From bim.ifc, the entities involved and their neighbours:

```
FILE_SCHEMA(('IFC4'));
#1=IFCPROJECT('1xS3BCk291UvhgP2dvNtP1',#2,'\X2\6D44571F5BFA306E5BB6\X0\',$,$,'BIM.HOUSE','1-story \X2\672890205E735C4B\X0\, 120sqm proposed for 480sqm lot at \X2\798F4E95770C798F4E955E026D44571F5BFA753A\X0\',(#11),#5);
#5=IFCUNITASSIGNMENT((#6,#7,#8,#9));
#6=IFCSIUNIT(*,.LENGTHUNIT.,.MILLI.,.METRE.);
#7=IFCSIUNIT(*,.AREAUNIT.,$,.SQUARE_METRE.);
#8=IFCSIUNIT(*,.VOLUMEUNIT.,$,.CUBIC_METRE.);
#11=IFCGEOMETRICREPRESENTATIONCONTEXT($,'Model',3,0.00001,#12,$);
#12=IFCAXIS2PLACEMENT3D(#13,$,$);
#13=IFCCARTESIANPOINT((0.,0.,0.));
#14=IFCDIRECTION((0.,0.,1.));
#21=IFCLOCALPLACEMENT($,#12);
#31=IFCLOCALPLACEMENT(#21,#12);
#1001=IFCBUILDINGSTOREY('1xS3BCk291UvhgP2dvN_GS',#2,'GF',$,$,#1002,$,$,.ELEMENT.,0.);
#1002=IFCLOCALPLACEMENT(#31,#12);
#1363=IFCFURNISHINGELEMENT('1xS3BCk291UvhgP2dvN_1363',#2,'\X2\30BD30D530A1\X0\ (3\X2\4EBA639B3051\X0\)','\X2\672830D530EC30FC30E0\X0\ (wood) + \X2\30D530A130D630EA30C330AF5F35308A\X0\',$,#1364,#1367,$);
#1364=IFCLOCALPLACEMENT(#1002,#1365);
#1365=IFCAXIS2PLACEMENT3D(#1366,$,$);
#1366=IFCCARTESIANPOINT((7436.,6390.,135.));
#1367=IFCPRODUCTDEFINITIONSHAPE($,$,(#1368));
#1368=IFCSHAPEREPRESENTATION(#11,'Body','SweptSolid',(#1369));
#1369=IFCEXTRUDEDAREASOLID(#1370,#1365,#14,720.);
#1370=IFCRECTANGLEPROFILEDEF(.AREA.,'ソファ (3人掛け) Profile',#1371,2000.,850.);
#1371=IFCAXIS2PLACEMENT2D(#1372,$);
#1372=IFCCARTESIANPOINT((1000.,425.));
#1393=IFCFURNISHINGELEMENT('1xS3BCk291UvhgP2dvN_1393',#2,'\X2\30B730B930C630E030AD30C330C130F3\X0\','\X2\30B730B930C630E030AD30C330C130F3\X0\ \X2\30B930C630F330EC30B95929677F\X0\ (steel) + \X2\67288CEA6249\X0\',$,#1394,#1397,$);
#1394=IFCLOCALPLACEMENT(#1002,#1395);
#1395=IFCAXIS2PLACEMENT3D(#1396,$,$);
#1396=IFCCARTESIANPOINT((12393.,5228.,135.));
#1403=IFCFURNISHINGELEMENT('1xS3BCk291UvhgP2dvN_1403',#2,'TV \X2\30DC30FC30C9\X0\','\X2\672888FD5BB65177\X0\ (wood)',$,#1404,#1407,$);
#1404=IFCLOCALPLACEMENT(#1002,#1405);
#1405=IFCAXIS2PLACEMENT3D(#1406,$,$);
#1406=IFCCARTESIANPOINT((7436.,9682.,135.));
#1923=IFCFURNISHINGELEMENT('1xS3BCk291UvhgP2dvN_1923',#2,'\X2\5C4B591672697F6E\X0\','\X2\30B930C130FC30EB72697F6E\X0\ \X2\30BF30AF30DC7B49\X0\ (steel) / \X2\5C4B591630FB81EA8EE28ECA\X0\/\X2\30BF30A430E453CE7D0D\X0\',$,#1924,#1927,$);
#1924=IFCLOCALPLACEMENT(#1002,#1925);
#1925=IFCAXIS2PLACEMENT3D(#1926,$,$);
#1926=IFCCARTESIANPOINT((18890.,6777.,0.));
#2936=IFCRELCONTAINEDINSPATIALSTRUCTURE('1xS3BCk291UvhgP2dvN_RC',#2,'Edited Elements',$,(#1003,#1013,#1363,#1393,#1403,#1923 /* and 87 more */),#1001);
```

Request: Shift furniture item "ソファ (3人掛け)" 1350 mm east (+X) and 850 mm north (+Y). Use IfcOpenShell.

```python
import ifcopenshell
import ifcopenshell.api.geometry
import ifcopenshell.util.placement
import ifcopenshell.util.unit

model = ifcopenshell.open("bim.ifc")
unit_scale = ifcopenshell.util.unit.calculate_unit_scale(model)

item = model.by_guid("1xS3BCk291UvhgP2dvN_1363")
matrix = ifcopenshell.util.placement.get_local_placement(item.ObjectPlacement)
matrix[0, 3] += 1.35 / unit_scale
matrix[1, 3] += 0.85 / unit_scale
ifcopenshell.api.geometry.edit_object_placement(model, product=item, matrix=matrix, is_si=False)

print(ifcopenshell.util.placement.get_local_placement(item.ObjectPlacement).round(3) + 0.0)

model.write("bim-out.ifc")
```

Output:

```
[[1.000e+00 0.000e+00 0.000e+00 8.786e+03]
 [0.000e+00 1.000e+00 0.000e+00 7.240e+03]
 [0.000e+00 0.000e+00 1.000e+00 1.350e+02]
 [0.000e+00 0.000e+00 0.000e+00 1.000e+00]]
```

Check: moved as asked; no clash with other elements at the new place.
